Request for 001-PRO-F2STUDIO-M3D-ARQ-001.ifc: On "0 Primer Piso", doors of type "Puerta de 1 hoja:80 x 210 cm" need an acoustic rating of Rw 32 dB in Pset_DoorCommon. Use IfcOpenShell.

First a look at what the model holds.

```python
import ifcopenshell
import ifcopenshell.util.element

model = ifcopenshell.open("001-PRO-F2STUDIO-M3D-ARQ-001.ifc")
print(model.schema)
storey = next(s for s in model.by_type("IfcBuildingStorey") if s.Name == "0 Primer Piso")
doors = [e for e in ifcopenshell.util.element.get_decomposition(storey) if e.is_a("IfcDoor")]
seen = {}
for e in doors:
    element_type = ifcopenshell.util.element.get_type(e)
    key = (element_type.Name if element_type != e and element_type else None, ifcopenshell.util.element.get_pset(e, "Pset_DoorCommon", "AcousticRating"))
    seen[key] = seen.get(key, 0) + 1
for (name, value), count in sorted(seen.items(), key=str):
    print(count, "x", name, "|", value)
```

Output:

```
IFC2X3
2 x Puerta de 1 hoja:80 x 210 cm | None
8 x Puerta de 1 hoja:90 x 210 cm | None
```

```python
import ifcopenshell
import ifcopenshell.api.pset
import ifcopenshell.util.element

model = ifcopenshell.open("001-PRO-F2STUDIO-M3D-ARQ-001.ifc")

storey = next(s for s in model.by_type("IfcBuildingStorey") if s.Name == "0 Primer Piso")
doors = [e for e in ifcopenshell.util.element.get_decomposition(storey) if e.is_a("IfcDoor")]

count = 0
for e in doors:
    element_type = ifcopenshell.util.element.get_type(e)
    if element_type in (None, e) or element_type.Name != "Puerta de 1 hoja:80 x 210 cm":
        continue
    # add_pset returns the element's existing set when there is one.
    pset = ifcopenshell.api.pset.add_pset(model, product=e, name="Pset_DoorCommon")
    ifcopenshell.api.pset.edit_pset(model, pset=pset, properties={"AcousticRating": "Rw 32 dB"})
    count += 1

print(count, "doors updated")

model.write("001-PRO-F2STUDIO-M3D-ARQ-001_rev.ifc")
```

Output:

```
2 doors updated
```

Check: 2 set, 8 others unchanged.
